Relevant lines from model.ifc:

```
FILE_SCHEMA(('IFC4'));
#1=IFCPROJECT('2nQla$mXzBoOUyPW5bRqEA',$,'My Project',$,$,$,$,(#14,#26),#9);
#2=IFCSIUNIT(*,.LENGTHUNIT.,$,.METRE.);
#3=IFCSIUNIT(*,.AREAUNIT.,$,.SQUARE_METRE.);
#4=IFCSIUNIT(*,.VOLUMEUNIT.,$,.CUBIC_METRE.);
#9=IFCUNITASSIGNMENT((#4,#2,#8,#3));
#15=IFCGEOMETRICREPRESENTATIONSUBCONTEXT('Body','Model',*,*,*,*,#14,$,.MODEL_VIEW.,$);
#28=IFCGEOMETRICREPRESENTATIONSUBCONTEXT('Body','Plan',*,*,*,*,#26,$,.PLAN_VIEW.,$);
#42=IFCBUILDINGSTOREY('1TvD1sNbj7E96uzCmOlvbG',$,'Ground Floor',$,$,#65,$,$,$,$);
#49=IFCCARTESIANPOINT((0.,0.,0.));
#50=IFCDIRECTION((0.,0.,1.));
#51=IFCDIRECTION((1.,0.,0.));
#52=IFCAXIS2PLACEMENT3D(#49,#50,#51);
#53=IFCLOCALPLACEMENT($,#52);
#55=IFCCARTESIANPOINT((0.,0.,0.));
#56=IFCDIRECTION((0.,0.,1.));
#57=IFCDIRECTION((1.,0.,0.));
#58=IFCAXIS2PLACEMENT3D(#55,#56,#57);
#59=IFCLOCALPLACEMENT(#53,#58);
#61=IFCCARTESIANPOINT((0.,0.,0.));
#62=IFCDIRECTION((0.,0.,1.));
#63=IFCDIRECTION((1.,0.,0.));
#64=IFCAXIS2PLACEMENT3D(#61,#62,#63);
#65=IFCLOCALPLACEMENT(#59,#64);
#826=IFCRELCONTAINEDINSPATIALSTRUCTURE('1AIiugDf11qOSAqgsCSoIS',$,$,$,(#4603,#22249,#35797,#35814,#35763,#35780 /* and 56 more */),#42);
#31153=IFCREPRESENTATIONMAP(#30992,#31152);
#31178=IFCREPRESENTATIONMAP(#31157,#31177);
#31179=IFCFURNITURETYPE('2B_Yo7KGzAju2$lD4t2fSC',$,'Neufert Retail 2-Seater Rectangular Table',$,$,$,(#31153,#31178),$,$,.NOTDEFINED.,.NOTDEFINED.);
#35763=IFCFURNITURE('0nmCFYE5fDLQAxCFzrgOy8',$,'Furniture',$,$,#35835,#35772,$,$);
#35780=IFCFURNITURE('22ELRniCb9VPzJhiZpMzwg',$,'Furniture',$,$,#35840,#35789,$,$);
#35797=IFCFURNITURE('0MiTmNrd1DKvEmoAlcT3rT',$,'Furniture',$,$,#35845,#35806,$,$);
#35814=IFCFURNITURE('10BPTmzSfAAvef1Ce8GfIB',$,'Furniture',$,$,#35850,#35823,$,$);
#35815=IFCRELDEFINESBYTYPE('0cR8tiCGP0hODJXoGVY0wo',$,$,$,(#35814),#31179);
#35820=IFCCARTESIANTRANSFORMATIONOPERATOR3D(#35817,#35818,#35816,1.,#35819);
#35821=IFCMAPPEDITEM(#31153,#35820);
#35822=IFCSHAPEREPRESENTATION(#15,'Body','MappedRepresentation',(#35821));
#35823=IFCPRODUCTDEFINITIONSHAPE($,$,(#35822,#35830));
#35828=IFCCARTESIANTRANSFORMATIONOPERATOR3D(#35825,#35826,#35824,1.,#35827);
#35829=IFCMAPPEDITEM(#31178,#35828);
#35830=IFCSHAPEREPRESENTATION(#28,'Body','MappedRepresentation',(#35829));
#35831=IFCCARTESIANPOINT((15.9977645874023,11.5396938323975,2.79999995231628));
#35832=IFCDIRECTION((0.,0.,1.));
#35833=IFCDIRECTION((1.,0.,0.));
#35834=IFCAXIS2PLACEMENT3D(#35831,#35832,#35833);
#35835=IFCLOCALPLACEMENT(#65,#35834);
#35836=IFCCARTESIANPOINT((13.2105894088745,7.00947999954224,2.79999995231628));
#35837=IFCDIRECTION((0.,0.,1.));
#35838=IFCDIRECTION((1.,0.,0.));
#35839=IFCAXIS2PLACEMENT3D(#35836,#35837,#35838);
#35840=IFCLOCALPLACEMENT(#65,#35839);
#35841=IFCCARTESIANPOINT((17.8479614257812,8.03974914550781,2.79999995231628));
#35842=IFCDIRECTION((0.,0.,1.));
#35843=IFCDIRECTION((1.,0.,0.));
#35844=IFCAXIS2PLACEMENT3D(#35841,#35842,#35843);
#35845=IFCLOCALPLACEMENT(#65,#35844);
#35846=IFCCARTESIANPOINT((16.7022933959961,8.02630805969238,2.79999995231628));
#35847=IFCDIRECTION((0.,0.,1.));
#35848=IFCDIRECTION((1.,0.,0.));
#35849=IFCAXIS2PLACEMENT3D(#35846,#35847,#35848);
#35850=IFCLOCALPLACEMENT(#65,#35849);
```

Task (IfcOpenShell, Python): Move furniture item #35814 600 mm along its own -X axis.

```python
import ifcopenshell
import ifcopenshell.api.geometry
import ifcopenshell.util.placement

model = ifcopenshell.open("model.ifc")

item = model.by_guid("10BPTmzSfAAvef1Ce8GfIB")
matrix = ifcopenshell.util.placement.get_local_placement(item.ObjectPlacement)
matrix[:3, 3] -= matrix[:3, 0] * 0.6
ifcopenshell.api.geometry.edit_object_placement(model, product=item, matrix=matrix, is_si=False)

print(ifcopenshell.util.placement.get_local_placement(item.ObjectPlacement).round(3) + 0.0)

model.write("model_rev.ifc")
```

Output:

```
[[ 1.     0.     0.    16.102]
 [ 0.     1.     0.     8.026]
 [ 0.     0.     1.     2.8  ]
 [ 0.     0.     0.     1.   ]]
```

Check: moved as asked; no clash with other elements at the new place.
